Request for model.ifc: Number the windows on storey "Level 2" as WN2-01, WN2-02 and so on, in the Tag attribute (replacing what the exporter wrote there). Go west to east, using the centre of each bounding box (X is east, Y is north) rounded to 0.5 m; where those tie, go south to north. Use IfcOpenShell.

First a look at what the model holds.

```python
import ifcopenshell
import ifcopenshell.util.element
import ifcopenshell.util.placement

model = ifcopenshell.open("model.ifc")
print(model.schema)
storey = next(s for s in model.by_type("IfcBuildingStorey") if s.Name == "Level 2")
windows = [e for e in ifcopenshell.util.element.get_decomposition(storey) if e.is_a("IfcWindow")]
for e in sorted(windows, key=lambda e: e.id()):
    origin = ifcopenshell.util.placement.get_local_placement(e.ObjectPlacement)[:3, 3]
    print(e.id(), e.Tag, e.Name, origin.round(2) + 0.0, sep=" | ")
```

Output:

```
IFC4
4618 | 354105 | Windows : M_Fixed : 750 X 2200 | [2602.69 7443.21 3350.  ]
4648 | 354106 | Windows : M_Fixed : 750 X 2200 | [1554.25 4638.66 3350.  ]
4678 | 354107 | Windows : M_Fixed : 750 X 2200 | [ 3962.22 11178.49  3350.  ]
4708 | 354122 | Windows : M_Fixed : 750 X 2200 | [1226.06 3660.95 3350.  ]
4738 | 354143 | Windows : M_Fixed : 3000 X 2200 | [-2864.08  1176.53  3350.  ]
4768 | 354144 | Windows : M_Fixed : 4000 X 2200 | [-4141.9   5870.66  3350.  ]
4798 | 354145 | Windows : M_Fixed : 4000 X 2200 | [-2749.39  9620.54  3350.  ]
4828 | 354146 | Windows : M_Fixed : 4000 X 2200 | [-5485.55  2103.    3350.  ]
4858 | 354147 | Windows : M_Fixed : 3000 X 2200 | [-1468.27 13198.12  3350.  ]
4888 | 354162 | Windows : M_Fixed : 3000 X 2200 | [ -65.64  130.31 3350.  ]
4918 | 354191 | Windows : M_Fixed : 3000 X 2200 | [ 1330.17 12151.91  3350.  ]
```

```python
import ifcopenshell
import ifcopenshell.geom
import ifcopenshell.util.element
import ifcopenshell.util.shape

model = ifcopenshell.open("model.ifc")
settings = ifcopenshell.geom.settings()
settings.set("use-world-coords", True)


def centre(element):
    shape = ifcopenshell.geom.create_shape(settings, element)
    return ifcopenshell.util.shape.get_bbox_centroid(shape.geometry)


storey = next(s for s in model.by_type("IfcBuildingStorey") if s.Name == "Level 2")
windows = [e for e in ifcopenshell.util.element.get_decomposition(storey) if e.is_a("IfcWindow")]

# Insertion points can sit at a corner or the storey origin, so sort by the geometry (in metres).
centres = {e: centre(e) for e in windows}
windows.sort(key=lambda e: (round(centres[e][0] / 0.5), centres[e][1]))

for i, e in enumerate(windows, start=1):
    number = f"WN2-{i:02d}"
    e.Tag = number
    print(e.id(), number)

model.write("model-out.ifc")
```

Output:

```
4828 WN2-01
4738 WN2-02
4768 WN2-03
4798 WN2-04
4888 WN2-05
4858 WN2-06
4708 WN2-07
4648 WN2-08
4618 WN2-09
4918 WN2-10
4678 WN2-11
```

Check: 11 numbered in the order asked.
